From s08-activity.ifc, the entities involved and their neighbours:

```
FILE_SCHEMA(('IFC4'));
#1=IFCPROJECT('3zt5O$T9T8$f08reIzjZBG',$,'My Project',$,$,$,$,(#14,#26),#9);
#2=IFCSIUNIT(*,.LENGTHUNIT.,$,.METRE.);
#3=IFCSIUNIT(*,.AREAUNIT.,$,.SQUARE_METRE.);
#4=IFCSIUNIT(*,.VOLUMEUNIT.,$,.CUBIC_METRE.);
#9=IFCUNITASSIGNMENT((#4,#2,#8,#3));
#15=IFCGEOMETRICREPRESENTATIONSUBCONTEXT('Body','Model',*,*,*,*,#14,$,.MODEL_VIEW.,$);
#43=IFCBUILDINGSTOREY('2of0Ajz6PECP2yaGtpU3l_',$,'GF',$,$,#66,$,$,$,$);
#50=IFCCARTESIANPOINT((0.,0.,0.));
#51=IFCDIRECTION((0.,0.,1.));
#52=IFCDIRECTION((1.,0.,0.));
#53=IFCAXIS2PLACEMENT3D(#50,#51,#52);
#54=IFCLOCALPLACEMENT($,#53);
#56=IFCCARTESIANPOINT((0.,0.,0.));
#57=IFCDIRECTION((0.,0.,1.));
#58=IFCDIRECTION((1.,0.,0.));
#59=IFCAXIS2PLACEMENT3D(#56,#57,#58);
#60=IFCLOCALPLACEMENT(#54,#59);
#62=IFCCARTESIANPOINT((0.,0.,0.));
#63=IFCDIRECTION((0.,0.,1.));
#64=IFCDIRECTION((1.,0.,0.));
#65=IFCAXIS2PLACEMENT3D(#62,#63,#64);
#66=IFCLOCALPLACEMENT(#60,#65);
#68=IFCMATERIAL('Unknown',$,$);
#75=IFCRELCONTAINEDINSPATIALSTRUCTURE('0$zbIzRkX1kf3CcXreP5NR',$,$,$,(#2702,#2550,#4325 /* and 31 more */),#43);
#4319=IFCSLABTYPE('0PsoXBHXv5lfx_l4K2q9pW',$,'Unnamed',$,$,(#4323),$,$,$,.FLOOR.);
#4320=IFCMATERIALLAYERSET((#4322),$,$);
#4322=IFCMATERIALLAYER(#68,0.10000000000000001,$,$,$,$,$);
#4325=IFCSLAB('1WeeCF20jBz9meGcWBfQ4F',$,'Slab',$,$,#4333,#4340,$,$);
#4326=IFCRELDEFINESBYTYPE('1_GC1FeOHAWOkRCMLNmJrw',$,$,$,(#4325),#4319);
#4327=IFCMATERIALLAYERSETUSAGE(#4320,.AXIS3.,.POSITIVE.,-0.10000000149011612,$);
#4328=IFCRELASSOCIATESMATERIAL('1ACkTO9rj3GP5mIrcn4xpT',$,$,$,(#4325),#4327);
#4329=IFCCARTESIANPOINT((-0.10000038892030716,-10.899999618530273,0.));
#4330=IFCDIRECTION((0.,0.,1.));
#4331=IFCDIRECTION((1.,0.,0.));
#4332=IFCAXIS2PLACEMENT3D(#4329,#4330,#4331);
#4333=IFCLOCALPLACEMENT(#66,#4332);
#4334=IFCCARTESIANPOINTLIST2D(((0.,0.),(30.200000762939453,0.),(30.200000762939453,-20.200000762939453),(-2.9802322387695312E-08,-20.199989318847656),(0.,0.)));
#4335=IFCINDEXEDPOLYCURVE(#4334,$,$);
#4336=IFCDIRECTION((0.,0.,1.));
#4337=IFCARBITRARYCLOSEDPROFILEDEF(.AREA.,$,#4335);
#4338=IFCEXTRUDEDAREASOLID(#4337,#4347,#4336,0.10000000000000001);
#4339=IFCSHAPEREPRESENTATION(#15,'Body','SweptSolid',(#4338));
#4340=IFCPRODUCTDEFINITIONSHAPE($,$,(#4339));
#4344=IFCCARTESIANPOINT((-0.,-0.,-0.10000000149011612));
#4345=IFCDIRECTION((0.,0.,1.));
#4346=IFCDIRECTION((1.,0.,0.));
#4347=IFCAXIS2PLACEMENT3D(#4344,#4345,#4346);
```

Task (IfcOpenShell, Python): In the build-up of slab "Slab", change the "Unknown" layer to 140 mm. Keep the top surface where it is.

```python
import ifcopenshell
import ifcopenshell.util.element
import ifcopenshell.util.representation
import ifcopenshell.util.unit

model = ifcopenshell.open("s08-activity.ifc")
unit_scale = ifcopenshell.util.unit.calculate_unit_scale(model)

layer_set = model.by_id(4320)
layer = next(l for l in layer_set.MaterialLayers if l.Material and l.Material.Name == "Unknown")
change = 0.14 / unit_scale - layer.LayerThickness
layer.LayerThickness += change

# Geometry does not follow the layer set by itself.
slabs = [e for e in ifcopenshell.util.element.get_elements_by_material(model, layer_set) if e.is_a("IfcSlab")]
for slab in sorted(slabs, key=lambda e: e.id()):
    body = ifcopenshell.util.representation.get_representation(slab, "Model", "Body")
    solid = body.Items[0]
    old_depth = solid.Depth
    solid.Depth += change
    # Extruded upwards: lower the start of the extrusion so the top stays.
    x, y, z = solid.Position.Location.Coordinates
    solid.Position.Location = model.createIfcCartesianPoint((x, y, z - change))
    print(slab.id(), f"{old_depth:g} -> {solid.Depth:g}")

# The layers are counted up from the underside, which has moved.
for usage in {ifcopenshell.util.element.get_material(slab) for slab in slabs}:
    usage.OffsetFromReferenceLine -= change

model.write("s08-activity_rev.ifc")
```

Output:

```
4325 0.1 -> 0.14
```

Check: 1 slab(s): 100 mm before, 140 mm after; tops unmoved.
